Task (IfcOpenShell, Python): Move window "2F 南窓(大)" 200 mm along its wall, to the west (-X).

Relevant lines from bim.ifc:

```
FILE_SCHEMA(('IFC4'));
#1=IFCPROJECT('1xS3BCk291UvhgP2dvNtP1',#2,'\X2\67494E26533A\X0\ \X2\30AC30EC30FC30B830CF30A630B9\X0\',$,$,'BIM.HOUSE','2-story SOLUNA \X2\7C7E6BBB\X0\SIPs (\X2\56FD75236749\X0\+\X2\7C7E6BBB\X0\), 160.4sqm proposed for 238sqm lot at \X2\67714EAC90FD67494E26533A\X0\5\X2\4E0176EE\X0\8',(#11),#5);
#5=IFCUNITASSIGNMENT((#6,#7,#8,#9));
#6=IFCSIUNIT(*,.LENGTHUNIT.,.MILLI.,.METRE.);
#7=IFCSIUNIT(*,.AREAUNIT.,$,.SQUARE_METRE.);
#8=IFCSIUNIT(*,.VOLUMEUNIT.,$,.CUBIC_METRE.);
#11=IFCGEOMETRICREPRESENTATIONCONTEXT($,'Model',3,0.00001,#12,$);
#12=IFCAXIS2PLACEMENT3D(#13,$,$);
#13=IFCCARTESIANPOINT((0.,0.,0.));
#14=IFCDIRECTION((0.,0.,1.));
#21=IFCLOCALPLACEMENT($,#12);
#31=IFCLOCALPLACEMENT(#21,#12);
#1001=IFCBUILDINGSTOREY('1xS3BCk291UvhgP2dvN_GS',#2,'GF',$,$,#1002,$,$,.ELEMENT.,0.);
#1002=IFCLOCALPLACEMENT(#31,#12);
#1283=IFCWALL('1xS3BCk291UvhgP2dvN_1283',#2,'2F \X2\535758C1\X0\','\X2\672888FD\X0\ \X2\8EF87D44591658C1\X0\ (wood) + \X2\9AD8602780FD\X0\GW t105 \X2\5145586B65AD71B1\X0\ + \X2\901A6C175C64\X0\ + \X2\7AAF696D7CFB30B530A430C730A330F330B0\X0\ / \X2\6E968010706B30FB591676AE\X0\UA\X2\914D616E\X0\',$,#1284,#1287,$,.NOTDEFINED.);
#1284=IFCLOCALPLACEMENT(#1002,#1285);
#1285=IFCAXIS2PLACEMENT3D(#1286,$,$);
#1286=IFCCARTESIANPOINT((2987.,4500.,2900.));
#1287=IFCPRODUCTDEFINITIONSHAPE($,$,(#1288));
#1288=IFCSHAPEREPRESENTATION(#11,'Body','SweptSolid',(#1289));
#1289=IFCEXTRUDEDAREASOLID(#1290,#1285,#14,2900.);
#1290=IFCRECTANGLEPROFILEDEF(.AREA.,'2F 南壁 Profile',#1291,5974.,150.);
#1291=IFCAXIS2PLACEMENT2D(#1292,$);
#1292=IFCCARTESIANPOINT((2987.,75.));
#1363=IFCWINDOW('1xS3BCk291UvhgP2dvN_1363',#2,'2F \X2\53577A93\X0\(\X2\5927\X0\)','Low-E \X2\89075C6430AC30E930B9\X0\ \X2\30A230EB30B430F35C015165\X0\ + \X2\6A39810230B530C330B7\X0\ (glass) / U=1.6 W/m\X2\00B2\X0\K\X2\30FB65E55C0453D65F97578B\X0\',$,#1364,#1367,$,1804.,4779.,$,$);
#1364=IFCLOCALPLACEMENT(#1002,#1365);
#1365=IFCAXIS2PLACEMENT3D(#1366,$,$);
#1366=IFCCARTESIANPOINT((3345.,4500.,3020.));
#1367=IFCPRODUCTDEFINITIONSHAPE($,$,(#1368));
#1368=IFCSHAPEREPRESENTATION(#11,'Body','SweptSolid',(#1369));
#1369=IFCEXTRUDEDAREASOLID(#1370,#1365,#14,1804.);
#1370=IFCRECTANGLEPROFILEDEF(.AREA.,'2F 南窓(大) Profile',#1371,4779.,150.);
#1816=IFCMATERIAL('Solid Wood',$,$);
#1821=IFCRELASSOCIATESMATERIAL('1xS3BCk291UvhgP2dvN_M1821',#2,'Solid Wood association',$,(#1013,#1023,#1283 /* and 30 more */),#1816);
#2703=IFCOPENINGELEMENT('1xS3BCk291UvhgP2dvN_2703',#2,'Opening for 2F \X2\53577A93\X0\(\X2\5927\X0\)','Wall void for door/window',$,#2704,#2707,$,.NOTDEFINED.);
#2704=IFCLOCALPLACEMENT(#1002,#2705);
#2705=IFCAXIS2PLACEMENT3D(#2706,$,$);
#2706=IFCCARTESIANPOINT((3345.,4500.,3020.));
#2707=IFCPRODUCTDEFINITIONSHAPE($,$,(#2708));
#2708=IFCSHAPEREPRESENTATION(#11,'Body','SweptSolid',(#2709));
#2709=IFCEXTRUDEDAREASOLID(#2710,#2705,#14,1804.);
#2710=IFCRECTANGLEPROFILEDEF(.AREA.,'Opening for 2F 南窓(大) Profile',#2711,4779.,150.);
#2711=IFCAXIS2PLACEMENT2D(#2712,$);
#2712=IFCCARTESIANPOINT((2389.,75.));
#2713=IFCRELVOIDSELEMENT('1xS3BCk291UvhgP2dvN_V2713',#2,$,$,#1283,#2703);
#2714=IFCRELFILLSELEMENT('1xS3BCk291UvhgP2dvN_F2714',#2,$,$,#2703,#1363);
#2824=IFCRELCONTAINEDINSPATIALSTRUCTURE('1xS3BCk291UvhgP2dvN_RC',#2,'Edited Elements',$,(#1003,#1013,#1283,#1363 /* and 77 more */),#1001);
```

```python
import ifcopenshell
import ifcopenshell.api.geometry
import ifcopenshell.util.placement
import ifcopenshell.util.unit

model = ifcopenshell.open("bim.ifc")
unit_scale = ifcopenshell.util.unit.calculate_unit_scale(model)

window = model.by_guid("1xS3BCk291UvhgP2dvN_1363")
opening = window.FillsVoids[0].RelatingOpeningElement
wall = opening.VoidsElements[0].RelatingBuildingElement

wall_matrix = ifcopenshell.util.placement.get_local_placement(wall.ObjectPlacement)
shift = wall_matrix[:3, 0] * -0.2 / unit_scale
before = ifcopenshell.util.placement.get_local_placement(window.ObjectPlacement)[:3, 3].copy()

# The window is not placed relative to its opening, so move both.
for product in (opening, window):
    matrix = ifcopenshell.util.placement.get_local_placement(product.ObjectPlacement)
    matrix[:3, 3] += shift
    ifcopenshell.api.geometry.edit_object_placement(model, product=product, matrix=matrix, is_si=False)

after = ifcopenshell.util.placement.get_local_placement(window.ObjectPlacement)[:3, 3]
print("window moved by", (after - before).round(3) + 0.0)

model.write("bim_rev.ifc")
```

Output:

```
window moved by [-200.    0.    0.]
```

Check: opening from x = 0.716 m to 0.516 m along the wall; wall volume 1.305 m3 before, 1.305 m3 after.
